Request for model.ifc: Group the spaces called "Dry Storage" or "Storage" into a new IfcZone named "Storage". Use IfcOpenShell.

First a look at what the model holds.

```python
import ifcopenshell

model = ifcopenshell.open("model.ifc")
print(model.schema)
seen = {}
for space in model.by_type("IfcSpace"):
    seen[space.LongName] = seen.get(space.LongName, 0) + 1
for name, count in sorted(seen.items(), key=str):
    print(count, "x", name)
print("zones:", [z.Name for z in model.by_type("IfcZone")][:20])
```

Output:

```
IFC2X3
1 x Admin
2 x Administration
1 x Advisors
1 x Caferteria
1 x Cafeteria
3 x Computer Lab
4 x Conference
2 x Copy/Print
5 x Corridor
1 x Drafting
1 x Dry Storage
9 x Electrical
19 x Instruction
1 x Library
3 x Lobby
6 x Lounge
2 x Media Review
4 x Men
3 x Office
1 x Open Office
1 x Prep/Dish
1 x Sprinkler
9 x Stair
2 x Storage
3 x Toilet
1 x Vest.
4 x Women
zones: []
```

```python
import ifcopenshell
import ifcopenshell.api.group
import ifcopenshell.api.root

model = ifcopenshell.open("model.ifc")

names = {"Dry Storage", "Storage"}
spaces = [s for s in model.by_type("IfcSpace") if s.LongName in names]

zone = ifcopenshell.api.root.create_entity(model, ifc_class="IfcZone", name="Storage")
ifcopenshell.api.group.assign_group(model, products=spaces, group=zone)
print(len(spaces), "spaces in", zone.Name)

model.write("model_rev.ifc")
```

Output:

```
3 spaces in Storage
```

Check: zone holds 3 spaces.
